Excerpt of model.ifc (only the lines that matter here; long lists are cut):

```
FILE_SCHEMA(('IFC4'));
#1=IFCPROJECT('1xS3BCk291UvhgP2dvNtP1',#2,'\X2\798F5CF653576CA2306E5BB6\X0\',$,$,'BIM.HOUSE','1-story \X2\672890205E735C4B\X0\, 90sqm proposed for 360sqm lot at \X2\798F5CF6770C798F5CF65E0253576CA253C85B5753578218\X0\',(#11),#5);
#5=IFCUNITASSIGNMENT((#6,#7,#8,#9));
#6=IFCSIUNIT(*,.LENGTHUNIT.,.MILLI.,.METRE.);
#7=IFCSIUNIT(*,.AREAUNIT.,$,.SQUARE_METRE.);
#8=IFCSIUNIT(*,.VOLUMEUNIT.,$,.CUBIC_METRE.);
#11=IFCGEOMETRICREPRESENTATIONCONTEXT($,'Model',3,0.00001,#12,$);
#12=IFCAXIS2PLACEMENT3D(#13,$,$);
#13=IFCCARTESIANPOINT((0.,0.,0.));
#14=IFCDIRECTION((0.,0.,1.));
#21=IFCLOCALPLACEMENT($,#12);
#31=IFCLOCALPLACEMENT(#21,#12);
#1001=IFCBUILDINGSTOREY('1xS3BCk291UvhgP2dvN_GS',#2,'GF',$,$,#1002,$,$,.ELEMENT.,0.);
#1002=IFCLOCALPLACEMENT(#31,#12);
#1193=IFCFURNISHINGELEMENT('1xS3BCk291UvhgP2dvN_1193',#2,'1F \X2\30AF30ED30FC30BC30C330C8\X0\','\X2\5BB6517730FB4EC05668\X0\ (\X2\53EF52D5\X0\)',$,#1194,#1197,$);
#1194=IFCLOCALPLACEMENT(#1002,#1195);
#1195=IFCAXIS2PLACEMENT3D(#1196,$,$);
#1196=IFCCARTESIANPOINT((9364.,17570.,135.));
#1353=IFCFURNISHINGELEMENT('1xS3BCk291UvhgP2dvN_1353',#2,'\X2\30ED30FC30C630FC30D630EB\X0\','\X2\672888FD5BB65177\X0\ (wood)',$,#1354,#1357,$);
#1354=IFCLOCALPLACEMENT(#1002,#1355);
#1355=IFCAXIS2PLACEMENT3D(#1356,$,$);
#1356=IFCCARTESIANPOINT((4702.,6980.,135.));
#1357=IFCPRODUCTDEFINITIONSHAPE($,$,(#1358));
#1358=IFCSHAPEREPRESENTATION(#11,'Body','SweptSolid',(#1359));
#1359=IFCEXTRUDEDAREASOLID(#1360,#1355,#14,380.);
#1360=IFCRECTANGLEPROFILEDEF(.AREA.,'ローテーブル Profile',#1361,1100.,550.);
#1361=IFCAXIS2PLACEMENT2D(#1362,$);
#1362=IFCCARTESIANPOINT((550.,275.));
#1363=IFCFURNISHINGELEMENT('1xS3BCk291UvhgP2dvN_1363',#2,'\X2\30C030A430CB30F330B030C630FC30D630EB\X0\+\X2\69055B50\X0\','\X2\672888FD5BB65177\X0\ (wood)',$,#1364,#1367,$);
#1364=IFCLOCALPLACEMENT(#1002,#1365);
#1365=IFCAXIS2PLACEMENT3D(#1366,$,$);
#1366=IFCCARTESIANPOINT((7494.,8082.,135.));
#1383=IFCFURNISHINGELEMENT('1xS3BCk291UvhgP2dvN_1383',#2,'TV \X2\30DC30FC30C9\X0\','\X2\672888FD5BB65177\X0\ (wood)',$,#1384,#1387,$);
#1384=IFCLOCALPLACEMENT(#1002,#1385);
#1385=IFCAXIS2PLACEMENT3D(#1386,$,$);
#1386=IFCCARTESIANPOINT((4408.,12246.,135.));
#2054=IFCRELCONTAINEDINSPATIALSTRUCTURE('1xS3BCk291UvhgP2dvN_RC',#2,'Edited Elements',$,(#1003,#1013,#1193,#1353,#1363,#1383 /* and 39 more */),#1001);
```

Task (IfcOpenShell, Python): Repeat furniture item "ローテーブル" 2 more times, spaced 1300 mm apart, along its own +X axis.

```python
import ifcopenshell
import ifcopenshell.api.geometry
import ifcopenshell.api.root
import ifcopenshell.util.element
import ifcopenshell.util.placement
import ifcopenshell.util.unit

model = ifcopenshell.open("model.ifc")
unit_scale = ifcopenshell.util.unit.calculate_unit_scale(model)


def reuse_history(source, copy):
    """copy_class also copies each property set's owner history, people and application; keep the originals."""
    for rel in copy.IsDefinedBy:
        if rel.is_a("IfcRelDefinesByProperties") and (history := rel.RelatingPropertyDefinition.OwnerHistory):
            rel.RelatingPropertyDefinition.OwnerHistory = source.OwnerHistory
            ifcopenshell.util.element.remove_deep2(model, history)


source = model.by_guid("1xS3BCk291UvhgP2dvN_1353")
base = ifcopenshell.util.placement.get_local_placement(source.ObjectPlacement)
step = base[:3, 0] * 1.3 / unit_scale

for i in range(1, 3):
    copy = ifcopenshell.api.root.copy_class(model, product=source)
    copy.Representation = ifcopenshell.util.element.copy_deep(
        model, source.Representation, exclude=["IfcGeometricRepresentationContext", "IfcRepresentationMap"]
    )
    reuse_history(source, copy)
    matrix = base.copy()
    matrix[:3, 3] += i * step
    print("added at", matrix[:3, 3].round(3) + 0.0)
    ifcopenshell.api.geometry.edit_object_placement(model, product=copy, matrix=matrix, is_si=False)

model.write("model_updated.ifc")
```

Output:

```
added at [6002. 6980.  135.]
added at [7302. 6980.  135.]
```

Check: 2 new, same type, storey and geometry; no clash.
